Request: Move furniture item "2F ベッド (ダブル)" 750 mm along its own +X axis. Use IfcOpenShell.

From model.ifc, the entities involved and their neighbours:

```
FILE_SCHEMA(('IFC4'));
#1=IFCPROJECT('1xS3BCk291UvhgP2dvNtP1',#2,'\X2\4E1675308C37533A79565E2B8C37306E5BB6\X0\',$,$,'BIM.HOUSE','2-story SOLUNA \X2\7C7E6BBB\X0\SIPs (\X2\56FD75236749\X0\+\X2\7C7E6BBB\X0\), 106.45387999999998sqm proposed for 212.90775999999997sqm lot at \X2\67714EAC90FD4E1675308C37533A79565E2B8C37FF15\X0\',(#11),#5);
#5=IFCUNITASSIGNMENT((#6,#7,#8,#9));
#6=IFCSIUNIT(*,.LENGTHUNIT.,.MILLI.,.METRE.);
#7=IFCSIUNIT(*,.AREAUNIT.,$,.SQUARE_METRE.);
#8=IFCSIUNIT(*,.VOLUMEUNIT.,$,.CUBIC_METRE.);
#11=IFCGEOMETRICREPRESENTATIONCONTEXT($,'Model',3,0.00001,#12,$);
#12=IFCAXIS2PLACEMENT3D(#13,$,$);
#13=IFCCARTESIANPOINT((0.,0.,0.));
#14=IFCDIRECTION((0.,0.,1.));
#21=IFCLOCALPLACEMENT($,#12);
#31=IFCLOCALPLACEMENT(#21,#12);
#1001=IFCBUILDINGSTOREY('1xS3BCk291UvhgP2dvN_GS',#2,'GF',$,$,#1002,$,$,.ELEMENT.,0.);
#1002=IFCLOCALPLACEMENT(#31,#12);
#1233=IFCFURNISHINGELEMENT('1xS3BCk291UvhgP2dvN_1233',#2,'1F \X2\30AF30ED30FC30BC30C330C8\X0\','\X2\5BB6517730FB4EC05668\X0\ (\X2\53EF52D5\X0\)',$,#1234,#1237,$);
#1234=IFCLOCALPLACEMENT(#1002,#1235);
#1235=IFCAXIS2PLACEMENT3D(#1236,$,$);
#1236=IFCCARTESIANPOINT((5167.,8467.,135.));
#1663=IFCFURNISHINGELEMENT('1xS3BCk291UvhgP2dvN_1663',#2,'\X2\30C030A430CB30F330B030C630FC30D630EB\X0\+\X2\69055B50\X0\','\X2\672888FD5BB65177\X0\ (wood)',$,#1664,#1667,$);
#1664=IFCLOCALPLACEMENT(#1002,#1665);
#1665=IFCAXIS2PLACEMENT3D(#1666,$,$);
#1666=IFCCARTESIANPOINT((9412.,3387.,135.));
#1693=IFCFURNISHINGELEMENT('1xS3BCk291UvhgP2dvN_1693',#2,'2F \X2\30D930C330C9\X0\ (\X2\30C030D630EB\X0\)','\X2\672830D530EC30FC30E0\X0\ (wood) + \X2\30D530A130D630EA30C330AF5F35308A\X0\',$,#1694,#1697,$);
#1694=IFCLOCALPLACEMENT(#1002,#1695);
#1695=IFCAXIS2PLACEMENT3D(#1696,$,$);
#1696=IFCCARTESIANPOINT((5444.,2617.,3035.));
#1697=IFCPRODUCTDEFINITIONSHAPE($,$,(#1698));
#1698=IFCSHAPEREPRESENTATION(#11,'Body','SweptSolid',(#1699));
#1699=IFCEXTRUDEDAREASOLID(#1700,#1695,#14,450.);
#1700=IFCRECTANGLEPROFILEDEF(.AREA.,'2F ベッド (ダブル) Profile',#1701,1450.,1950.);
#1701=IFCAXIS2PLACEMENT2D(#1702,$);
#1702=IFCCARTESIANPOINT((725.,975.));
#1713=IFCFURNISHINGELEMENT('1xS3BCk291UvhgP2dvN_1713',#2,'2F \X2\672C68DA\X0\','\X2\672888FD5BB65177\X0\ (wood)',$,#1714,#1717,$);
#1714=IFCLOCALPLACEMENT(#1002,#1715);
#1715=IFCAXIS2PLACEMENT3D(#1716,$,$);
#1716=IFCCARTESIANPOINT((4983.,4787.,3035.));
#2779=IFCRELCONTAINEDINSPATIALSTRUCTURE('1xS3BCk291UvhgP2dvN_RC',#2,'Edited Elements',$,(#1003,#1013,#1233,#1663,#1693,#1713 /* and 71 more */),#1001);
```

```python
import ifcopenshell
import ifcopenshell.api.geometry
import ifcopenshell.util.placement

model = ifcopenshell.open("model.ifc")

item = model.by_guid("1xS3BCk291UvhgP2dvN_1693")
matrix = ifcopenshell.util.placement.get_local_placement(item.ObjectPlacement)
matrix[:3, 3] += matrix[:3, 0] * 750.0
ifcopenshell.api.geometry.edit_object_placement(model, product=item, matrix=matrix, is_si=False)

print(ifcopenshell.util.placement.get_local_placement(item.ObjectPlacement).round(3) + 0.0)

model.write("model_v2.ifc")
```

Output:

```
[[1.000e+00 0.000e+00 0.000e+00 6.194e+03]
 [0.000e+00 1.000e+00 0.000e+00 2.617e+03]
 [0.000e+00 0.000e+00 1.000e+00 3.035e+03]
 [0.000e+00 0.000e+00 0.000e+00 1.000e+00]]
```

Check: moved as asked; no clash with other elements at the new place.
